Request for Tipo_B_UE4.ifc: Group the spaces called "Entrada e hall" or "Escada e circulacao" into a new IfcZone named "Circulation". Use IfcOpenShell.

First a look at what the model holds.

```python
import ifcopenshell

model = ifcopenshell.open("Tipo_B_UE4.ifc")
print(model.schema)
seen = {}
for space in model.by_type("IfcSpace"):
    seen[space.Name] = seen.get(space.Name, 0) + 1
for name, count in sorted(seen.items(), key=str):
    print(count, "x", name)
print("zones:", [z.Name for z in model.by_type("IfcZone")][:20])
```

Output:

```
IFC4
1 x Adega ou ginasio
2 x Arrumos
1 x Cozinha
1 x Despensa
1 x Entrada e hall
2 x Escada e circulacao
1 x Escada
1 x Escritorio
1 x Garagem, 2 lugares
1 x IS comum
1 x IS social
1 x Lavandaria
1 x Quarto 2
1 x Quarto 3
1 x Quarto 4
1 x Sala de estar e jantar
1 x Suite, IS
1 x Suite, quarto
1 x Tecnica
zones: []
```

```python
import ifcopenshell
import ifcopenshell.api.group
import ifcopenshell.api.root

model = ifcopenshell.open("Tipo_B_UE4.ifc")

names = {"Entrada e hall", "Escada e circulacao"}
spaces = [s for s in model.by_type("IfcSpace") if s.Name in names]

zone = ifcopenshell.api.root.create_entity(model, ifc_class="IfcZone", name="Circulation")
ifcopenshell.api.group.assign_group(model, products=spaces, group=zone)
print(len(spaces), "spaces in", zone.Name)

model.write("Tipo_B_UE4_rev.ifc")
```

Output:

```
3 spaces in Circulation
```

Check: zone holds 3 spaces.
